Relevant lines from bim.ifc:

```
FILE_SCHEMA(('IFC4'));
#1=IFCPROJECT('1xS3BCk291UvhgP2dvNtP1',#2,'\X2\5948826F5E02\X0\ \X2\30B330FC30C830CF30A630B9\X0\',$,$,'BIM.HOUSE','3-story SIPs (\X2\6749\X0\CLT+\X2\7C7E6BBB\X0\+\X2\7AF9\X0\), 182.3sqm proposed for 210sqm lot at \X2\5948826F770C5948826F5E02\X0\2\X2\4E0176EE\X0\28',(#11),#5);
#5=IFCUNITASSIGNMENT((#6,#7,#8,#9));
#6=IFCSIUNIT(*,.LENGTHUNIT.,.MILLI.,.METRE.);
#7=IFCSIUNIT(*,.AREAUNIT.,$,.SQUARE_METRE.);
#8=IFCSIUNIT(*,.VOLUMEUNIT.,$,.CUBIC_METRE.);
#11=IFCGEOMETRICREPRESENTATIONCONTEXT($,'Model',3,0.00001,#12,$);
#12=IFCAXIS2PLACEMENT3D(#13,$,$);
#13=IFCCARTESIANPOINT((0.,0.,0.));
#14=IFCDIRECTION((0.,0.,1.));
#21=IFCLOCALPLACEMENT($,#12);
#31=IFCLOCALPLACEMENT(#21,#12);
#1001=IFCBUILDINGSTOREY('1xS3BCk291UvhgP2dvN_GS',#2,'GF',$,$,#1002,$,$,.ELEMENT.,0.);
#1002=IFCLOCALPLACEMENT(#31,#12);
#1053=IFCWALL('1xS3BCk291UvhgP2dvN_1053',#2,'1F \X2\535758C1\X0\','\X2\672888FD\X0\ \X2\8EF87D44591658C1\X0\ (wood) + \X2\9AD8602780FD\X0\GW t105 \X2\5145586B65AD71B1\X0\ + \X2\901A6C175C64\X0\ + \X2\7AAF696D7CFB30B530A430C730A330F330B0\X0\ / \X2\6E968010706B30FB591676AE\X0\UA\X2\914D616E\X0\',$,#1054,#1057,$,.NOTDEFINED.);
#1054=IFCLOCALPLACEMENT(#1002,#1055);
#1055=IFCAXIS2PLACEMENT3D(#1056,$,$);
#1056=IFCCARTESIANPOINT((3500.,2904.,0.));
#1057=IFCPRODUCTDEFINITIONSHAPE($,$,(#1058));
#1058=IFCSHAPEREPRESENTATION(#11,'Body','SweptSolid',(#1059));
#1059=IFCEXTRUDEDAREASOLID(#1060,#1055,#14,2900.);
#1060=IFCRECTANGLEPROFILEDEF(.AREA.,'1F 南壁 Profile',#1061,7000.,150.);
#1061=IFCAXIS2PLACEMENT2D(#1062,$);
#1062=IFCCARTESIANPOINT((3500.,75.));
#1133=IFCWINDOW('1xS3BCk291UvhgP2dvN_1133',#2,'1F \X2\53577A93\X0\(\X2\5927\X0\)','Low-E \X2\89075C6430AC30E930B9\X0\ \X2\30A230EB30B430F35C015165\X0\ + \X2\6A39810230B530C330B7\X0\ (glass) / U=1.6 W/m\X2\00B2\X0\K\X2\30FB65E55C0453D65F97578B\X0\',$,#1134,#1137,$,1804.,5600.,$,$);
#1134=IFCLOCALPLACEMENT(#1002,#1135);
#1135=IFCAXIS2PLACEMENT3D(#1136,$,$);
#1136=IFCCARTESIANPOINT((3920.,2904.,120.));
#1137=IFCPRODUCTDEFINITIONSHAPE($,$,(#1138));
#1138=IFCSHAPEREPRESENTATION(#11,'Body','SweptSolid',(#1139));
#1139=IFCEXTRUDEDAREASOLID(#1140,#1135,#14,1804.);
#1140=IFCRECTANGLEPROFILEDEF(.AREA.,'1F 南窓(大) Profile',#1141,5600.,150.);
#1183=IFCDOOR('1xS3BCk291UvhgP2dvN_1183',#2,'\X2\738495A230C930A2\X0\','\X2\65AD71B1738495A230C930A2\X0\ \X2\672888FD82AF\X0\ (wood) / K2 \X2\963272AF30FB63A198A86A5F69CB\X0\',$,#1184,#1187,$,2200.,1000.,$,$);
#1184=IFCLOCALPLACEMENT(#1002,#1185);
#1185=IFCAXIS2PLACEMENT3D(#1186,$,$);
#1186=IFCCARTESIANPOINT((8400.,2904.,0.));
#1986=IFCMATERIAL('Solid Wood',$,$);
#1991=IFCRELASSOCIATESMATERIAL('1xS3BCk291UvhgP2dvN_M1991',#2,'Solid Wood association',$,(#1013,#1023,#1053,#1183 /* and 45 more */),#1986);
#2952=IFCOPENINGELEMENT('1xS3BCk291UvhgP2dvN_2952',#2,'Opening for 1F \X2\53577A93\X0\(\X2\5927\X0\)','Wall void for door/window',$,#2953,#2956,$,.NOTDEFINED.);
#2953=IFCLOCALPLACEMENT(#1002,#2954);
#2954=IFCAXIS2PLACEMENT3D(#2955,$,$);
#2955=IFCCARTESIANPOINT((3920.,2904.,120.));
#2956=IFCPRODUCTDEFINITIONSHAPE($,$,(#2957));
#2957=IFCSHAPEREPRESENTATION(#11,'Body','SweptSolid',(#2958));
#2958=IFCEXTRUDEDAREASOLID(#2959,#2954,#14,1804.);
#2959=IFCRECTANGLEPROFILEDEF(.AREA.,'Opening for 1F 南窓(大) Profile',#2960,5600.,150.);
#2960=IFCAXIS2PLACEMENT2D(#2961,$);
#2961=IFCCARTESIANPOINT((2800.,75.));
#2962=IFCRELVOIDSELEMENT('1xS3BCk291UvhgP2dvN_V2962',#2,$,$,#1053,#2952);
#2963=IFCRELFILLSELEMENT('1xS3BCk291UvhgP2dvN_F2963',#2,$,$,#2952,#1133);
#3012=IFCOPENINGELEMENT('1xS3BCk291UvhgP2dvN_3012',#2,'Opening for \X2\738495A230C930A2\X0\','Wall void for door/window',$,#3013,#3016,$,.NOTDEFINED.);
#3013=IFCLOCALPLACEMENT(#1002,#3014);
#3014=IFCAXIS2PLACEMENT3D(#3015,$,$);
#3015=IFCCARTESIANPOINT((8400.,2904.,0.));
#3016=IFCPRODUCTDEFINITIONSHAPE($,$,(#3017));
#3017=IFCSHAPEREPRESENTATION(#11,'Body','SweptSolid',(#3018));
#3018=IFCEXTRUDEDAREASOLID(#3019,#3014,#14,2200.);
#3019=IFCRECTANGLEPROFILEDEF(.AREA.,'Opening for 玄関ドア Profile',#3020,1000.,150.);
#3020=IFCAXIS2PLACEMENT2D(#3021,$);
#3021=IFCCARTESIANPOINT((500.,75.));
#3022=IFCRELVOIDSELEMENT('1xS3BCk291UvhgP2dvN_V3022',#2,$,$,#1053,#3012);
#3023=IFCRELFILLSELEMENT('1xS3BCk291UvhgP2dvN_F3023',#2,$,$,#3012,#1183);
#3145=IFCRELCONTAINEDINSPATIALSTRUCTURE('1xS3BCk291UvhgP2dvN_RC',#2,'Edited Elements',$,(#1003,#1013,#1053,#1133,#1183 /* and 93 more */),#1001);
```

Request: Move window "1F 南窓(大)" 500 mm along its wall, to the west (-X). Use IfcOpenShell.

```python
import ifcopenshell
import ifcopenshell.api.geometry
import ifcopenshell.util.placement
import ifcopenshell.util.unit

model = ifcopenshell.open("bim.ifc")
unit_scale = ifcopenshell.util.unit.calculate_unit_scale(model)

window = model.by_guid("1xS3BCk291UvhgP2dvN_1133")
opening = window.FillsVoids[0].RelatingOpeningElement
wall = opening.VoidsElements[0].RelatingBuildingElement

wall_matrix = ifcopenshell.util.placement.get_local_placement(wall.ObjectPlacement)
shift = wall_matrix[:3, 0] * -0.5 / unit_scale
before = ifcopenshell.util.placement.get_local_placement(window.ObjectPlacement)[:3, 3].copy()

# The window is not placed relative to its opening, so move both.
for product in (opening, window):
    matrix = ifcopenshell.util.placement.get_local_placement(product.ObjectPlacement)
    matrix[:3, 3] += shift
    ifcopenshell.api.geometry.edit_object_placement(model, product=product, matrix=matrix, is_si=False)

after = ifcopenshell.util.placement.get_local_placement(window.ObjectPlacement)[:3, 3]
print("window moved by", (after - before).round(3) + 0.0)

model.write("bim_updated.ifc")
```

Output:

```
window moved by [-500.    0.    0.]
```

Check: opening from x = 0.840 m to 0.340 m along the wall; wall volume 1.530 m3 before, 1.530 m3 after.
